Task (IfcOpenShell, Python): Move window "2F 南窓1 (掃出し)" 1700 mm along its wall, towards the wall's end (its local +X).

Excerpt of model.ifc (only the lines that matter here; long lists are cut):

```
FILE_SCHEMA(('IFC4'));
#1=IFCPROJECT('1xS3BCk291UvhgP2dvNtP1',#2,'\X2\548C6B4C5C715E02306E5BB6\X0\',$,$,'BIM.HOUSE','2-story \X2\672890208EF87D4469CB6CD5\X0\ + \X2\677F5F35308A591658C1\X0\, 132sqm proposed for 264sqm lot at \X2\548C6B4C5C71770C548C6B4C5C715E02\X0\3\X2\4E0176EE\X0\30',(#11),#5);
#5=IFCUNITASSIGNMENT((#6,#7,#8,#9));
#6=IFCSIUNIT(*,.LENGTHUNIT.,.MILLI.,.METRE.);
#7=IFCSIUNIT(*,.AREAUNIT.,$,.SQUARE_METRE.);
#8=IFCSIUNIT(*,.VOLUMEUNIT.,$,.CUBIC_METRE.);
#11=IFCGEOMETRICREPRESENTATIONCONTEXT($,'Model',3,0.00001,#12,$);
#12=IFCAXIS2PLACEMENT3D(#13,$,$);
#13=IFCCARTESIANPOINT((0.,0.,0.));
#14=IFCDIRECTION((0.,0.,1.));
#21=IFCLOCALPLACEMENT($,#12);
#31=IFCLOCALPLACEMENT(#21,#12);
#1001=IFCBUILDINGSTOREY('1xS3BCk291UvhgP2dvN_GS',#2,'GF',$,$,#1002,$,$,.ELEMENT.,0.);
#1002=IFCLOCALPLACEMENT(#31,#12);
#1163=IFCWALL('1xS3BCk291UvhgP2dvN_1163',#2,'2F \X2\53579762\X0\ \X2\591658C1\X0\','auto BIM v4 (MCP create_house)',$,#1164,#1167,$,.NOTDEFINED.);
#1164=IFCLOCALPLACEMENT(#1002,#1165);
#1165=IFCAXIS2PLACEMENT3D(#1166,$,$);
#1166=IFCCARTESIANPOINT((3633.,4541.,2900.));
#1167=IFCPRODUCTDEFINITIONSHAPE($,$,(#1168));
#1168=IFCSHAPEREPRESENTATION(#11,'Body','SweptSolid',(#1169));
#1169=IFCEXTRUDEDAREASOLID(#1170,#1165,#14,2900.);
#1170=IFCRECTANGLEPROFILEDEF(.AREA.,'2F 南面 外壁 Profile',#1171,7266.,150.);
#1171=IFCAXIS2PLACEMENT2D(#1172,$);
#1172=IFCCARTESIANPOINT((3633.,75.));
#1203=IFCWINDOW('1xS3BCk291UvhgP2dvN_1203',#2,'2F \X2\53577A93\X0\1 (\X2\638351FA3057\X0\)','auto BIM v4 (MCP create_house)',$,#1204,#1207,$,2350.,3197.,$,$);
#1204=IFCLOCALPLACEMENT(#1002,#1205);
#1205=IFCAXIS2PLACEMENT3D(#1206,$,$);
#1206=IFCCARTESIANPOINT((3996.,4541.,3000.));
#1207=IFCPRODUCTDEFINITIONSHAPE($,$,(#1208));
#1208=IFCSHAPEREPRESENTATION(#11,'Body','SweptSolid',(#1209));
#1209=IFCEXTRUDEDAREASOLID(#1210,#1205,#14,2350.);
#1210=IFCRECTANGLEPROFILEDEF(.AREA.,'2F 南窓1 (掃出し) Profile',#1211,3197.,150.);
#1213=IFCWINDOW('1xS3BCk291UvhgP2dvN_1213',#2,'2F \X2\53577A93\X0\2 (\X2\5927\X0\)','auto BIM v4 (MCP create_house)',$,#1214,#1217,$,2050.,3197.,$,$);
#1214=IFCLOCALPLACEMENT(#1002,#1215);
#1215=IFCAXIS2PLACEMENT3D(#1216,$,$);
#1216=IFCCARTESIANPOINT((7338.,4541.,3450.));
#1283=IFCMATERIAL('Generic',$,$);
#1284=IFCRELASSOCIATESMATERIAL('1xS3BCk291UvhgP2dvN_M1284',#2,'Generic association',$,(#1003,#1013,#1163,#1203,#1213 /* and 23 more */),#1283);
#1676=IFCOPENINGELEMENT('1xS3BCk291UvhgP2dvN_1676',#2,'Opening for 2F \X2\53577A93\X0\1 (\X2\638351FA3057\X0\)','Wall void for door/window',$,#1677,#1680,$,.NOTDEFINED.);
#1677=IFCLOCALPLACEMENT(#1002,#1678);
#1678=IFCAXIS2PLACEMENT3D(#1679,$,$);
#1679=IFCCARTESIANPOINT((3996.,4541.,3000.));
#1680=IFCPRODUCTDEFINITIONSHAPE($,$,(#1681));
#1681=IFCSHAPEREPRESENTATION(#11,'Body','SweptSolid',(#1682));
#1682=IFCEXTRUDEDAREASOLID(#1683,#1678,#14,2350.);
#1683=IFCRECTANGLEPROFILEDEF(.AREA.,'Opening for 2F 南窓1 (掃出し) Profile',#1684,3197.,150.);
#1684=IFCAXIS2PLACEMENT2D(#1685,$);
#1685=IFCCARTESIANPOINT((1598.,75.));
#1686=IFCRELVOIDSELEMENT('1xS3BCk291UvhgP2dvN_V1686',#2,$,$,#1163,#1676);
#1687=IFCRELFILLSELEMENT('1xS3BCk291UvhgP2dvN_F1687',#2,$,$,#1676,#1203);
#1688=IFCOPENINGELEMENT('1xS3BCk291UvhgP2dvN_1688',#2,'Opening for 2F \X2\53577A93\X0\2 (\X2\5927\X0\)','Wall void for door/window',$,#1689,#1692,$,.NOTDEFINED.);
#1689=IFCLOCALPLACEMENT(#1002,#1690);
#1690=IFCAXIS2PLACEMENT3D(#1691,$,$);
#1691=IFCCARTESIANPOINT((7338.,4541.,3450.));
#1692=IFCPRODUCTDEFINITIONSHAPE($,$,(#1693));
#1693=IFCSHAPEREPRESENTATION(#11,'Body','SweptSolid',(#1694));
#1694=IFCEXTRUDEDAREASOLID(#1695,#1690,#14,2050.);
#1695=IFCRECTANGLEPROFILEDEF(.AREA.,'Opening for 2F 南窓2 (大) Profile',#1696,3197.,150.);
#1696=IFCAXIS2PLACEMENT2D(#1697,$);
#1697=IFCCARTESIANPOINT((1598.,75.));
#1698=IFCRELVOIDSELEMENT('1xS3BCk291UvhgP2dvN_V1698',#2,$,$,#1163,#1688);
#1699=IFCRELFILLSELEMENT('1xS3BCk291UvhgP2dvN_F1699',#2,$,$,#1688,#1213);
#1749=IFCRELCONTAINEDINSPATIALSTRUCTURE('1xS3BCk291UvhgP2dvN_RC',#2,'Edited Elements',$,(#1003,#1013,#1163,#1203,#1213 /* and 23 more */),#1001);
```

```python
import ifcopenshell
import ifcopenshell.api.geometry
import ifcopenshell.util.placement
import ifcopenshell.util.unit

model = ifcopenshell.open("model.ifc")
unit_scale = ifcopenshell.util.unit.calculate_unit_scale(model)

window = model.by_guid("1xS3BCk291UvhgP2dvN_1203")
opening = window.FillsVoids[0].RelatingOpeningElement
wall = opening.VoidsElements[0].RelatingBuildingElement

wall_matrix = ifcopenshell.util.placement.get_local_placement(wall.ObjectPlacement)
shift = wall_matrix[:3, 0] * 1.7 / unit_scale
before = ifcopenshell.util.placement.get_local_placement(window.ObjectPlacement)[:3, 3].copy()

# The window is not placed relative to its opening, so move both.
for product in (opening, window):
    matrix = ifcopenshell.util.placement.get_local_placement(product.ObjectPlacement)
    matrix[:3, 3] += shift
    ifcopenshell.api.geometry.edit_object_placement(model, product=product, matrix=matrix, is_si=False)

after = ifcopenshell.util.placement.get_local_placement(window.ObjectPlacement)[:3, 3]
print("window moved by", (after - before).round(3) + 0.0)

model.write("model_updated.ifc")
```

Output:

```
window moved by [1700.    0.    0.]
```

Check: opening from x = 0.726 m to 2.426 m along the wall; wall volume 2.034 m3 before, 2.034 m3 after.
